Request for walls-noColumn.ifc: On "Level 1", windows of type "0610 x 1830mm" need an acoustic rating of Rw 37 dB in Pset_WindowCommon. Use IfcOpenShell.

First a look at what the model holds.

```python
import ifcopenshell
import ifcopenshell.util.element

model = ifcopenshell.open("walls-noColumn.ifc")
print(model.schema)
storey = next(s for s in model.by_type("IfcBuildingStorey") if s.Name == "Level 1")
windows = [e for e in ifcopenshell.util.element.get_decomposition(storey) if e.is_a("IfcWindow")]
seen = {}
for e in windows:
    element_type = ifcopenshell.util.element.get_type(e)
    key = (element_type.Name if element_type != e and element_type else None, ifcopenshell.util.element.get_pset(e, "Pset_WindowCommon", "AcousticRating"))
    seen[key] = seen.get(key, 0) + 1
for (name, value), count in sorted(seen.items(), key=str):
    print(count, "x", name, "|", value)
```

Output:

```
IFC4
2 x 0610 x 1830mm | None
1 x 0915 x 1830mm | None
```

```python
import ifcopenshell
import ifcopenshell.api.pset
import ifcopenshell.util.element

model = ifcopenshell.open("walls-noColumn.ifc")

storey = next(s for s in model.by_type("IfcBuildingStorey") if s.Name == "Level 1")
windows = [e for e in ifcopenshell.util.element.get_decomposition(storey) if e.is_a("IfcWindow")]

count = 0
for e in windows:
    element_type = ifcopenshell.util.element.get_type(e)
    if element_type in (None, e) or element_type.Name != "0610 x 1830mm":
        continue
    # add_pset returns the element's existing set when there is one.
    pset = ifcopenshell.api.pset.add_pset(model, product=e, name="Pset_WindowCommon")
    ifcopenshell.api.pset.edit_pset(model, pset=pset, properties={"AcousticRating": "Rw 37 dB"})
    count += 1

print(count, "windows updated")

model.write("walls-noColumn_edited.ifc")
```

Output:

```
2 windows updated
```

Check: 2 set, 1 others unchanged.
